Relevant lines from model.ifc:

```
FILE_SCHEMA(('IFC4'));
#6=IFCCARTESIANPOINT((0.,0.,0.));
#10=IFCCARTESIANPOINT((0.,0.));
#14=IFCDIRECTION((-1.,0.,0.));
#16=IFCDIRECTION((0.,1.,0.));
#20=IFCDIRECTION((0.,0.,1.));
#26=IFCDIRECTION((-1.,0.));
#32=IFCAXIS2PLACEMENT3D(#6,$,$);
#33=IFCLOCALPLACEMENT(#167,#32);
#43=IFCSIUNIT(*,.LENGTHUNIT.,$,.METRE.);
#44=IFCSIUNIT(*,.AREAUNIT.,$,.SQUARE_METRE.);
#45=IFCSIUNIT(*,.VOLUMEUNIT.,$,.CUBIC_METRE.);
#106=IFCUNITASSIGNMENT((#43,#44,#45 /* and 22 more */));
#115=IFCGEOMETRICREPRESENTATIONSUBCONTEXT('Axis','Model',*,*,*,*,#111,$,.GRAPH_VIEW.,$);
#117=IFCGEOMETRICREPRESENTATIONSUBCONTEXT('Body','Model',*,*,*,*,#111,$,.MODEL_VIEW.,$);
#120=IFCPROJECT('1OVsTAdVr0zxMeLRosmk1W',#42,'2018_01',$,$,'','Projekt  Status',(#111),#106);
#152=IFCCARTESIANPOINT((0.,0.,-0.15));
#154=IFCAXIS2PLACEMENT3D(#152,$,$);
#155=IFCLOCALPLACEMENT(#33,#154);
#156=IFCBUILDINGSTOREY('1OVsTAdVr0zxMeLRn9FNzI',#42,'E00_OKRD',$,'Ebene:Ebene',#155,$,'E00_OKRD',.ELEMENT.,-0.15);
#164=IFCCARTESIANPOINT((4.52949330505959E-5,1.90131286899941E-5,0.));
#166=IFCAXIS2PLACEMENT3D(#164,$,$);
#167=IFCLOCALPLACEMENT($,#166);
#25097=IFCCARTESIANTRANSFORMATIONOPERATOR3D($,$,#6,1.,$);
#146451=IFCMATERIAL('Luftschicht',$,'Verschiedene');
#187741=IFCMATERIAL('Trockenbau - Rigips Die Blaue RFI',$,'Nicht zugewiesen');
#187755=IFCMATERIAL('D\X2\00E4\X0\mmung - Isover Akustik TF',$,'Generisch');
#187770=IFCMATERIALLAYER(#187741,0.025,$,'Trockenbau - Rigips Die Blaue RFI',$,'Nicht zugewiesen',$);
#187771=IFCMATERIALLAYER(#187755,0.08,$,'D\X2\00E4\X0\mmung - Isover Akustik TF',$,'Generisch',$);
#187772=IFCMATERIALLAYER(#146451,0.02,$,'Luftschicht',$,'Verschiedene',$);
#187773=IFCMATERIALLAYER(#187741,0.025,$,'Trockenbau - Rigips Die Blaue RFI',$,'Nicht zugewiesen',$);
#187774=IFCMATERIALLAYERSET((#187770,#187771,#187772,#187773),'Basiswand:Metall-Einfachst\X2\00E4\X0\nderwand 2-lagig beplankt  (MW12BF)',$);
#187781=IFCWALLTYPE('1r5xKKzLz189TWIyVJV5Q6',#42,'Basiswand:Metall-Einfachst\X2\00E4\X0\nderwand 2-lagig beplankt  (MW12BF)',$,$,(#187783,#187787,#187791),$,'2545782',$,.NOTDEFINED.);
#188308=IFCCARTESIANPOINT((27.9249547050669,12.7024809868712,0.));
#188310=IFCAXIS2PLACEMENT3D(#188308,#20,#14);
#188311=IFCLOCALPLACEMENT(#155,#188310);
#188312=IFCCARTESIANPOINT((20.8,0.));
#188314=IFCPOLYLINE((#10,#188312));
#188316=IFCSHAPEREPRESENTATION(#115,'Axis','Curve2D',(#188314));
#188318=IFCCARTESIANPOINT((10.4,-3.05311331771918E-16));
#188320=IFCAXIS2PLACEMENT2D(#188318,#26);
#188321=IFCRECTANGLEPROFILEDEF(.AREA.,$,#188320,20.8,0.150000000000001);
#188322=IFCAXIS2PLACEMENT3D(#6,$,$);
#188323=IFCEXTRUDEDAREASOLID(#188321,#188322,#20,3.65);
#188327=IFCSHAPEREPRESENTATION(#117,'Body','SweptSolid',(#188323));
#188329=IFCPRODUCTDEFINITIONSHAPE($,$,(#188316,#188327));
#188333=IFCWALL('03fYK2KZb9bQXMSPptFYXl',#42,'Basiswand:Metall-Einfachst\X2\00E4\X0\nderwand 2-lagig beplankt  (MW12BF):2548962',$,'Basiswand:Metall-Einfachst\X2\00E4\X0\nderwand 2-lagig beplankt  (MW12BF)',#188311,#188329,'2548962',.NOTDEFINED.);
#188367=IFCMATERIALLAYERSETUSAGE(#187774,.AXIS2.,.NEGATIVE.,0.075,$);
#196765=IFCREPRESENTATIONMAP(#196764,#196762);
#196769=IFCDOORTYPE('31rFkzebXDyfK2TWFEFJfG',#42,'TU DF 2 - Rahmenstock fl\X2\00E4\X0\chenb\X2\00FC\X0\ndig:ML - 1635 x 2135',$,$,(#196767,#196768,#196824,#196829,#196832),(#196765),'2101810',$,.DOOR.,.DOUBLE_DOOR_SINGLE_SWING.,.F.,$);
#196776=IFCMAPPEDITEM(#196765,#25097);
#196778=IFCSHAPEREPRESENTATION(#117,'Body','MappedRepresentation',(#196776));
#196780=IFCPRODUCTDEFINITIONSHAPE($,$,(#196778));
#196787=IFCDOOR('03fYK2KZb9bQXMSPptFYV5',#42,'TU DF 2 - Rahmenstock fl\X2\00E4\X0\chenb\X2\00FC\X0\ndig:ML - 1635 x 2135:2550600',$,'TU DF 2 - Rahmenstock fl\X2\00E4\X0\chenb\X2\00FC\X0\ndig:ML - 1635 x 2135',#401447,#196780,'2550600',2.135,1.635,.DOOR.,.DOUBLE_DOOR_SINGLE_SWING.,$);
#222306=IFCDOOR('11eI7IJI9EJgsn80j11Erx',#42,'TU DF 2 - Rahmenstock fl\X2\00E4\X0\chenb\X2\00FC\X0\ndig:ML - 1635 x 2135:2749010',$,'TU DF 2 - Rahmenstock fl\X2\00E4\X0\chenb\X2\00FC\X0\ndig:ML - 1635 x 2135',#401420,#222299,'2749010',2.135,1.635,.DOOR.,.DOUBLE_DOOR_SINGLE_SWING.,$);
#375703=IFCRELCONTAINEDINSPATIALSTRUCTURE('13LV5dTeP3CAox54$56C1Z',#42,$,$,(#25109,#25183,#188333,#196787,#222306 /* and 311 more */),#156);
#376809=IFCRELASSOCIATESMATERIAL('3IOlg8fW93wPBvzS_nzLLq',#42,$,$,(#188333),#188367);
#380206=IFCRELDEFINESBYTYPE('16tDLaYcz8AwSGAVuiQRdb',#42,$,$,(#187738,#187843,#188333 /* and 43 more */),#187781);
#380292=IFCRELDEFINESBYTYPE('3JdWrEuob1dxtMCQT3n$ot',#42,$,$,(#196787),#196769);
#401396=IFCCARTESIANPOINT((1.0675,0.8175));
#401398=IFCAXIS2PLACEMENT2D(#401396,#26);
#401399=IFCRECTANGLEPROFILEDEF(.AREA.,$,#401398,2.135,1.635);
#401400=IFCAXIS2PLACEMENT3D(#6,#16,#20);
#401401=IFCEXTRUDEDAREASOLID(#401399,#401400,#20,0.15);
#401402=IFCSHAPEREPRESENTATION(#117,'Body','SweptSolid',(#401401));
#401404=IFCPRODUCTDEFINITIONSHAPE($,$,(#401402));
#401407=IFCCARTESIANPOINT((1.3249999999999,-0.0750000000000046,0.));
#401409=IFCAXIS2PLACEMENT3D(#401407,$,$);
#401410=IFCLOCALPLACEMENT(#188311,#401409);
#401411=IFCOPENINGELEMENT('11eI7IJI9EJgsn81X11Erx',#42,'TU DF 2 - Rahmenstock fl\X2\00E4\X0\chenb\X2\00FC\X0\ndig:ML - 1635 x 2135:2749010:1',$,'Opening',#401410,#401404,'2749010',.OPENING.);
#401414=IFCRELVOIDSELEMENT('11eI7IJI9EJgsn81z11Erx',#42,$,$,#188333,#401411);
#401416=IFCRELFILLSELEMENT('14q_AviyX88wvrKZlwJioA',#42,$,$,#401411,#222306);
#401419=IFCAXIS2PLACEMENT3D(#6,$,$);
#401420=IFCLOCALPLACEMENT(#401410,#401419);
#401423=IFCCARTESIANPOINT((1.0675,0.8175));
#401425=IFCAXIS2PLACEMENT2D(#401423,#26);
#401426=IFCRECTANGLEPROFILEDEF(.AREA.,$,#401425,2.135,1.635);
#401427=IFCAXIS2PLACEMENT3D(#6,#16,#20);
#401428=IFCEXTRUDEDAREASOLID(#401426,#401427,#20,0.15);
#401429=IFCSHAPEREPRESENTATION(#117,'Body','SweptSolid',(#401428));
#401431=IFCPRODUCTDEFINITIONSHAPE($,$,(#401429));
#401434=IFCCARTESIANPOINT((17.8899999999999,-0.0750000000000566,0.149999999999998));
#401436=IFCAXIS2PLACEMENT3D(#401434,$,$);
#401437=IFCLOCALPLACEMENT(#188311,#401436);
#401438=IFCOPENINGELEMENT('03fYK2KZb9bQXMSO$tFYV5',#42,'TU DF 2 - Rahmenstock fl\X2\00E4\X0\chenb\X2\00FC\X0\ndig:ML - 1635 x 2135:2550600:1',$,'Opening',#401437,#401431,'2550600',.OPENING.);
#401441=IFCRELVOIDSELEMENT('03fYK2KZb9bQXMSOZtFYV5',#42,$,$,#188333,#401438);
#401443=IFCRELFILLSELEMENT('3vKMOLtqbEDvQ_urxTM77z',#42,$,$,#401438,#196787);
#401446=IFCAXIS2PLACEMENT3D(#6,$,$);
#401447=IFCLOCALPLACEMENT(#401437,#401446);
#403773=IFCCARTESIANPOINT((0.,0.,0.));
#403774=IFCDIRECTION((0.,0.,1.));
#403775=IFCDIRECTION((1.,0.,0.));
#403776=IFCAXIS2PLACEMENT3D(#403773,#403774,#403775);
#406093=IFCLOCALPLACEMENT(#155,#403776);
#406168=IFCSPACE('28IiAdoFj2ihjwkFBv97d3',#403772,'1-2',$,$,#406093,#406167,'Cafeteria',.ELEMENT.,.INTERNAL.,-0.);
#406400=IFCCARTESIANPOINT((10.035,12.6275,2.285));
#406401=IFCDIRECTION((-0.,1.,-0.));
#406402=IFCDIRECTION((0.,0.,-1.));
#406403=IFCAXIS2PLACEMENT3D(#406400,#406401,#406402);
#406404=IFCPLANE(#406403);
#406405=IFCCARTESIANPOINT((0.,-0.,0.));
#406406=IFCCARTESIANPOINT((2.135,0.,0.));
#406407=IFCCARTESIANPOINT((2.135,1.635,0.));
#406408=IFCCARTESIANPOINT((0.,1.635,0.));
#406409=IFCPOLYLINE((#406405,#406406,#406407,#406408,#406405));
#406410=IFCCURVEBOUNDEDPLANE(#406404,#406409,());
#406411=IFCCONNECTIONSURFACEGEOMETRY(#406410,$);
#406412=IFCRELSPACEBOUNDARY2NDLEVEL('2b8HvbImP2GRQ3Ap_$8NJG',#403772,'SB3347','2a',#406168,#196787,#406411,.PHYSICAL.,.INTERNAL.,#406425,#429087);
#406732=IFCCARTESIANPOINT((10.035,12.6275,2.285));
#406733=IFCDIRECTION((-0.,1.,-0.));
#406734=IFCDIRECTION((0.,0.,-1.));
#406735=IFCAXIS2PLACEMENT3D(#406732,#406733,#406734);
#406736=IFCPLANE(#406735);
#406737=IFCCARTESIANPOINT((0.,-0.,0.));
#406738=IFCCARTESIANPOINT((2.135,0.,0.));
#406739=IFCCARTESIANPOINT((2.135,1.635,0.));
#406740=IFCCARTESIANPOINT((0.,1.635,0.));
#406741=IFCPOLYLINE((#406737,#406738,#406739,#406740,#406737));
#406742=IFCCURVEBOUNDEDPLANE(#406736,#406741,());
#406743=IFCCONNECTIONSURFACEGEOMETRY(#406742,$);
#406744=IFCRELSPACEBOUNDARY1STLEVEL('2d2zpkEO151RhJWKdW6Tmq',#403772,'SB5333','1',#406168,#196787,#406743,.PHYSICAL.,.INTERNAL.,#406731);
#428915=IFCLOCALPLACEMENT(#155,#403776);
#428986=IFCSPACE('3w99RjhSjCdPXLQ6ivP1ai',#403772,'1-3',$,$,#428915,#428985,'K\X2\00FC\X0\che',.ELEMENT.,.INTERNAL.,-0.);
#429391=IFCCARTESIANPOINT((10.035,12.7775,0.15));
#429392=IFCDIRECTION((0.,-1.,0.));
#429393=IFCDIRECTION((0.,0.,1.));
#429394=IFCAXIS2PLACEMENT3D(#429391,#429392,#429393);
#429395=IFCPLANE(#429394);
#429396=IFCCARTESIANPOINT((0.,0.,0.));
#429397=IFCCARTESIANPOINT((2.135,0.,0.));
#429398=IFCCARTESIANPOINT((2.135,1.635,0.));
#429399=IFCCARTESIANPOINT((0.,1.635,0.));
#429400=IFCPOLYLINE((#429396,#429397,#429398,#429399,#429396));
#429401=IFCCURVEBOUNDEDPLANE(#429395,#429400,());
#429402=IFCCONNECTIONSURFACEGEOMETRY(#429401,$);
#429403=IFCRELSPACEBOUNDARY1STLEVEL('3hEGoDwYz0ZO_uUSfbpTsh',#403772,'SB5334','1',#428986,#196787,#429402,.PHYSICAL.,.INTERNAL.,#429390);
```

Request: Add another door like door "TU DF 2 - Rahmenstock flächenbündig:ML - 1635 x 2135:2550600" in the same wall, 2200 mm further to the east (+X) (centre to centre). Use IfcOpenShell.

```python
import numpy as np
import ifcopenshell
import ifcopenshell.api.feature
import ifcopenshell.api.geometry
import ifcopenshell.api.root
import ifcopenshell.geom
import ifcopenshell.util.element
import ifcopenshell.util.placement
import ifcopenshell.util.shape
import ifcopenshell.util.unit

model = ifcopenshell.open("model.ifc")
unit_scale = ifcopenshell.util.unit.calculate_unit_scale(model)
settings = ifcopenshell.geom.settings()


def volume(element):
    """Net volume in cubic metres, openings subtracted."""
    shape = ifcopenshell.geom.create_shape(settings, element)
    return ifcopenshell.util.shape.get_volume(shape.geometry)


def reuse_history(source, copy):
    """copy_class also copies each property set's owner history, people and application; keep the originals."""
    for rel in copy.IsDefinedBy:
        if rel.is_a("IfcRelDefinesByProperties") and (history := rel.RelatingPropertyDefinition.OwnerHistory):
            rel.RelatingPropertyDefinition.OwnerHistory = source.OwnerHistory
            ifcopenshell.util.element.remove_deep2(model, history)


door = model.by_guid("03fYK2KZb9bQXMSPptFYV5")
opening = door.FillsVoids[0].RelatingOpeningElement
wall = opening.VoidsElements[0].RelatingBuildingElement
before = volume(wall)
shift = ifcopenshell.util.placement.get_local_placement(wall.ObjectPlacement)[:3, 0] * -2.2 / unit_scale

# copy_class copies the void relationship, type, container and properties, but no geometry.
new_opening = ifcopenshell.api.root.copy_class(model, product=opening)
new_opening.Representation = ifcopenshell.util.element.copy_deep(
    model, opening.Representation, exclude=["IfcGeometricRepresentationContext", "IfcRepresentationMap"]
)
new_opening.Name = "TU DF 2 - Rahmenstock flächenbündig:ML - 1635 x 2135"
new_opening.Tag = None
new_door = ifcopenshell.api.root.copy_class(model, product=door)
new_door.Representation = ifcopenshell.util.element.copy_deep(
    model, door.Representation, exclude=["IfcGeometricRepresentationContext", "IfcRepresentationMap"]
)
new_door.Name = "TU DF 2 - Rahmenstock flächenbündig:ML - 1635 x 2135"
new_door.Tag = None
reuse_history(door, new_door)
ifcopenshell.api.feature.add_filling(model, opening=new_opening, element=new_door)

for old, new in ((opening, new_opening), (door, new_door)):
    matrix = ifcopenshell.util.placement.get_local_placement(old.ObjectPlacement)
    matrix[:3, 3] += shift
    ifcopenshell.api.geometry.edit_object_placement(model, product=new, matrix=matrix, is_si=False)

# The copied space boundaries still share their surfaces with the original.
for rel in new_door.ProvidesBoundaries:
    if rel.ConnectionGeometry:
        rel.ConnectionGeometry = ifcopenshell.util.element.copy_deep(model, rel.ConnectionGeometry)

# Space boundary surfaces are stored in each space's coordinates; move them too.
for rel in new_door.ProvidesBoundaries:
    if not rel.ConnectionGeometry:
        continue
    surface = rel.ConnectionGeometry.SurfaceOnRelatingElement.BasisSurface
    space_matrix = ifcopenshell.util.placement.get_local_placement(rel.RelatingSpace.ObjectPlacement)
    point = np.array(surface.Position.Location.Coordinates) + space_matrix[:3, :3].T @ shift
    surface.Position = model.createIfcAxis2Placement3D(
        model.createIfcCartesianPoint(point.tolist()), surface.Position.Axis, surface.Position.RefDirection
    )

after = volume(wall)

print(f"wall volume {before:.3f} -> {after:.3f} m3")

model.write("model_edited.ifc")
```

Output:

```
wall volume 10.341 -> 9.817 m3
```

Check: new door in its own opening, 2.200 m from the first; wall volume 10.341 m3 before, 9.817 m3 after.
